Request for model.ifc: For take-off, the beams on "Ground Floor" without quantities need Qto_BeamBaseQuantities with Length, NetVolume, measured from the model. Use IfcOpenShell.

First a look at what the model holds.

```python
import ifcopenshell
import ifcopenshell.util.element
import ifcopenshell.util.unit

model = ifcopenshell.open("model.ifc")
print(model.schema)
for unit_type in ("LENGTHUNIT", "AREAUNIT", "VOLUMEUNIT"):
    print(unit_type, ifcopenshell.util.unit.calculate_unit_scale(model, unit_type))
storey = next(s for s in model.by_type("IfcBuildingStorey") if s.Name == "Ground Floor")
beams = [e for e in ifcopenshell.util.element.get_decomposition(storey) if e.is_a("IfcBeam")]
for e in sorted(beams, key=lambda e: e.id()):
    print(e.id(), e.is_a(), e.Name, list(ifcopenshell.util.element.get_psets(e, qtos_only=True)), sep=" | ")
```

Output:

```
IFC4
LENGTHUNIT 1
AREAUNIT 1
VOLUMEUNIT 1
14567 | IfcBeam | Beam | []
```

```python
import ifcopenshell
import ifcopenshell.api.pset
import ifcopenshell.geom
import ifcopenshell.util.element
import ifcopenshell.util.shape
import ifcopenshell.util.unit

model = ifcopenshell.open("model.ifc")
unit_scale = ifcopenshell.util.unit.calculate_unit_scale(model)
volume_scale = ifcopenshell.util.unit.calculate_unit_scale(model, "VOLUMEUNIT")
settings = ifcopenshell.geom.settings()

storey = next(s for s in model.by_type("IfcBuildingStorey") if s.Name == "Ground Floor")
beams = [e for e in ifcopenshell.util.element.get_decomposition(storey) if e.is_a("IfcBeam")]

for e in sorted(beams, key=lambda e: e.id()):
    if ifcopenshell.util.element.get_psets(e, qtos_only=True, should_inherit=False):
        continue
    # Geometry comes back in metres, in the element's own axes.
    shape = ifcopenshell.geom.create_shape(settings, e)
    values = {
        "Length": ifcopenshell.util.shape.get_max_xyz(shape.geometry) / unit_scale,
        "NetVolume": ifcopenshell.util.shape.get_volume(shape.geometry) / volume_scale,
    }
    qto = ifcopenshell.api.pset.add_qto(model, product=e, name="Qto_BeamBaseQuantities")
    ifcopenshell.api.pset.edit_qto(model, qto=qto, properties=values)
    print(e.id(), {k: round(v, 3) for k, v in values.items()})

model.write("model_edited.ifc")
```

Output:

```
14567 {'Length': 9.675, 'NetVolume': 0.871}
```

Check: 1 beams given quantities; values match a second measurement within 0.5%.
